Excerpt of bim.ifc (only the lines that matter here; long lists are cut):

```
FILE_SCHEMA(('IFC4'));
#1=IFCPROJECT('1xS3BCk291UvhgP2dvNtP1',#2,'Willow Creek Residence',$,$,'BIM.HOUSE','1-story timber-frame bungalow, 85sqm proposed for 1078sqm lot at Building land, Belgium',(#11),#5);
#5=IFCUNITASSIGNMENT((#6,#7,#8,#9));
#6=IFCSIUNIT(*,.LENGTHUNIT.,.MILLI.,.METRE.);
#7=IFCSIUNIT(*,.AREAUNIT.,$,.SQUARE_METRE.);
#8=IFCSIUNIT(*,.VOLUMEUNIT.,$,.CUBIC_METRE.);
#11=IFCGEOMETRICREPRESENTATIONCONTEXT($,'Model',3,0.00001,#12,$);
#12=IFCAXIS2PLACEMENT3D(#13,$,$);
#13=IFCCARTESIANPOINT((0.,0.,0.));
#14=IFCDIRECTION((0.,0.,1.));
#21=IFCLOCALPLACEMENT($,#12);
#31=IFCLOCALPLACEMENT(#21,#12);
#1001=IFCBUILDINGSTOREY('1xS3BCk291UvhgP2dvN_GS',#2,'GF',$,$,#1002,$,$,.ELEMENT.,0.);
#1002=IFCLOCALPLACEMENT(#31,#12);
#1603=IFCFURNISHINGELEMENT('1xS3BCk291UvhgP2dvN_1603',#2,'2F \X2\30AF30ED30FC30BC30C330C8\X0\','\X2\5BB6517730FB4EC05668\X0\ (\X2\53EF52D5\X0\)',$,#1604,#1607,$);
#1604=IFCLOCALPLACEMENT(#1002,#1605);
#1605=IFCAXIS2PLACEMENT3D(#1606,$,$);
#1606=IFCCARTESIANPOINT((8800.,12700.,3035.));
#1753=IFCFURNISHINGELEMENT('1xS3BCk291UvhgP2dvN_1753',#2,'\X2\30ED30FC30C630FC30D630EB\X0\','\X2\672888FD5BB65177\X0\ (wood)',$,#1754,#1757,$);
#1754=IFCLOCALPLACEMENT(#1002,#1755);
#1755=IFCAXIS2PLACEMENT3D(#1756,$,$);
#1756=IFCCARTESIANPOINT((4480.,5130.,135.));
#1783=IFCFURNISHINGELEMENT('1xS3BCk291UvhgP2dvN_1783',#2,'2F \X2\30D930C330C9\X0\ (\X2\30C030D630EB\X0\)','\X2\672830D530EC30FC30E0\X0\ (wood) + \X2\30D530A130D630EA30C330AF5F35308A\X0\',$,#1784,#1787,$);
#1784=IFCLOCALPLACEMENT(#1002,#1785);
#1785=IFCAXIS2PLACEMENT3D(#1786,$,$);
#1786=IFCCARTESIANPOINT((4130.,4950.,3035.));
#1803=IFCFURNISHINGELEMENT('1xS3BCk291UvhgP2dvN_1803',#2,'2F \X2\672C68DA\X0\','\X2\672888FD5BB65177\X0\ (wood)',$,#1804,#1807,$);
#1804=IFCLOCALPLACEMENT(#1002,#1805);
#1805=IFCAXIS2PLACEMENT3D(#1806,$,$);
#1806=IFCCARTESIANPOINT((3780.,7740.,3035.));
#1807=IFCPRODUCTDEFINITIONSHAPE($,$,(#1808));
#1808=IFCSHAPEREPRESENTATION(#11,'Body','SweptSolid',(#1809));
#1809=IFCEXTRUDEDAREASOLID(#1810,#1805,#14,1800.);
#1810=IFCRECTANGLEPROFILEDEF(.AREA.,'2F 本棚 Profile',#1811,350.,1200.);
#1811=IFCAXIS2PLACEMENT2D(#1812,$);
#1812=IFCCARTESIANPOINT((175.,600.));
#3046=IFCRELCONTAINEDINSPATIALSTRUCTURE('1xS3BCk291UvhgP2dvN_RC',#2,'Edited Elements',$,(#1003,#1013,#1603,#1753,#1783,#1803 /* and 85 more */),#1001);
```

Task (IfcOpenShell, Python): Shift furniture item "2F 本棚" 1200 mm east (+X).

```python
import ifcopenshell
import ifcopenshell.api.geometry
import ifcopenshell.util.placement

model = ifcopenshell.open("bim.ifc")

item = model.by_id(1803)
matrix = ifcopenshell.util.placement.get_local_placement(item.ObjectPlacement)
matrix[0, 3] += 1200.0
ifcopenshell.api.geometry.edit_object_placement(model, product=item, matrix=matrix, is_si=False)

print(ifcopenshell.util.placement.get_local_placement(item.ObjectPlacement).round(3) + 0.0)

model.write("bim_edited.ifc")
```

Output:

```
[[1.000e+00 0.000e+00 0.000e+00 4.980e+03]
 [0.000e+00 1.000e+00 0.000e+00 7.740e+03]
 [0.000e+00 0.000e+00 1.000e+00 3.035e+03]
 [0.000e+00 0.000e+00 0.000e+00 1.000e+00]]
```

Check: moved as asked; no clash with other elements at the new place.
